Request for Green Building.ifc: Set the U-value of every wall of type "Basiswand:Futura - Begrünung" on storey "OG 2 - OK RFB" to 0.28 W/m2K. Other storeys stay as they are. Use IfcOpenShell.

First a look at what the model holds.

```python
import ifcopenshell
import ifcopenshell.util.element

model = ifcopenshell.open("Green Building.ifc")
print(model.schema)
storey = next(s for s in model.by_type("IfcBuildingStorey") if s.Name == "OG 2 - OK RFB")
walls = [e for e in ifcopenshell.util.element.get_decomposition(storey) if e.is_a("IfcWall")]
seen = {}
for e in walls:
    element_type = ifcopenshell.util.element.get_type(e)
    key = (element_type.Name if element_type != e and element_type else None, ifcopenshell.util.element.get_pset(e, "Pset_WallCommon", "ThermalTransmittance"))
    seen[key] = seen.get(key, 0) + 1
for (name, value), count in sorted(seen.items(), key=str):
    print(count, "x", name, "|", value)
```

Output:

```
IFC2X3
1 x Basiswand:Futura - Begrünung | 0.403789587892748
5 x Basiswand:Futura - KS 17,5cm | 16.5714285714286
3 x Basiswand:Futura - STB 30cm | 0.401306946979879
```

```python
import ifcopenshell
import ifcopenshell.api.pset
import ifcopenshell.util.element

model = ifcopenshell.open("Green Building.ifc")

storey = next(s for s in model.by_type("IfcBuildingStorey") if s.Name == "OG 2 - OK RFB")
walls = [e for e in ifcopenshell.util.element.get_decomposition(storey) if e.is_a("IfcWall")]

count = 0
for e in walls:
    element_type = ifcopenshell.util.element.get_type(e)
    if element_type in (None, e) or element_type.Name != "Basiswand:Futura - Begrünung":
        continue
    # add_pset returns the element's existing set when there is one.
    pset = ifcopenshell.api.pset.add_pset(model, product=e, name="Pset_WallCommon")
    ifcopenshell.api.pset.edit_pset(model, pset=pset, properties={"ThermalTransmittance": 0.28})
    count += 1

print(count, "walls updated")

model.write("Green Building_v2.ifc")
```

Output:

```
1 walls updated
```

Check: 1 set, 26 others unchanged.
